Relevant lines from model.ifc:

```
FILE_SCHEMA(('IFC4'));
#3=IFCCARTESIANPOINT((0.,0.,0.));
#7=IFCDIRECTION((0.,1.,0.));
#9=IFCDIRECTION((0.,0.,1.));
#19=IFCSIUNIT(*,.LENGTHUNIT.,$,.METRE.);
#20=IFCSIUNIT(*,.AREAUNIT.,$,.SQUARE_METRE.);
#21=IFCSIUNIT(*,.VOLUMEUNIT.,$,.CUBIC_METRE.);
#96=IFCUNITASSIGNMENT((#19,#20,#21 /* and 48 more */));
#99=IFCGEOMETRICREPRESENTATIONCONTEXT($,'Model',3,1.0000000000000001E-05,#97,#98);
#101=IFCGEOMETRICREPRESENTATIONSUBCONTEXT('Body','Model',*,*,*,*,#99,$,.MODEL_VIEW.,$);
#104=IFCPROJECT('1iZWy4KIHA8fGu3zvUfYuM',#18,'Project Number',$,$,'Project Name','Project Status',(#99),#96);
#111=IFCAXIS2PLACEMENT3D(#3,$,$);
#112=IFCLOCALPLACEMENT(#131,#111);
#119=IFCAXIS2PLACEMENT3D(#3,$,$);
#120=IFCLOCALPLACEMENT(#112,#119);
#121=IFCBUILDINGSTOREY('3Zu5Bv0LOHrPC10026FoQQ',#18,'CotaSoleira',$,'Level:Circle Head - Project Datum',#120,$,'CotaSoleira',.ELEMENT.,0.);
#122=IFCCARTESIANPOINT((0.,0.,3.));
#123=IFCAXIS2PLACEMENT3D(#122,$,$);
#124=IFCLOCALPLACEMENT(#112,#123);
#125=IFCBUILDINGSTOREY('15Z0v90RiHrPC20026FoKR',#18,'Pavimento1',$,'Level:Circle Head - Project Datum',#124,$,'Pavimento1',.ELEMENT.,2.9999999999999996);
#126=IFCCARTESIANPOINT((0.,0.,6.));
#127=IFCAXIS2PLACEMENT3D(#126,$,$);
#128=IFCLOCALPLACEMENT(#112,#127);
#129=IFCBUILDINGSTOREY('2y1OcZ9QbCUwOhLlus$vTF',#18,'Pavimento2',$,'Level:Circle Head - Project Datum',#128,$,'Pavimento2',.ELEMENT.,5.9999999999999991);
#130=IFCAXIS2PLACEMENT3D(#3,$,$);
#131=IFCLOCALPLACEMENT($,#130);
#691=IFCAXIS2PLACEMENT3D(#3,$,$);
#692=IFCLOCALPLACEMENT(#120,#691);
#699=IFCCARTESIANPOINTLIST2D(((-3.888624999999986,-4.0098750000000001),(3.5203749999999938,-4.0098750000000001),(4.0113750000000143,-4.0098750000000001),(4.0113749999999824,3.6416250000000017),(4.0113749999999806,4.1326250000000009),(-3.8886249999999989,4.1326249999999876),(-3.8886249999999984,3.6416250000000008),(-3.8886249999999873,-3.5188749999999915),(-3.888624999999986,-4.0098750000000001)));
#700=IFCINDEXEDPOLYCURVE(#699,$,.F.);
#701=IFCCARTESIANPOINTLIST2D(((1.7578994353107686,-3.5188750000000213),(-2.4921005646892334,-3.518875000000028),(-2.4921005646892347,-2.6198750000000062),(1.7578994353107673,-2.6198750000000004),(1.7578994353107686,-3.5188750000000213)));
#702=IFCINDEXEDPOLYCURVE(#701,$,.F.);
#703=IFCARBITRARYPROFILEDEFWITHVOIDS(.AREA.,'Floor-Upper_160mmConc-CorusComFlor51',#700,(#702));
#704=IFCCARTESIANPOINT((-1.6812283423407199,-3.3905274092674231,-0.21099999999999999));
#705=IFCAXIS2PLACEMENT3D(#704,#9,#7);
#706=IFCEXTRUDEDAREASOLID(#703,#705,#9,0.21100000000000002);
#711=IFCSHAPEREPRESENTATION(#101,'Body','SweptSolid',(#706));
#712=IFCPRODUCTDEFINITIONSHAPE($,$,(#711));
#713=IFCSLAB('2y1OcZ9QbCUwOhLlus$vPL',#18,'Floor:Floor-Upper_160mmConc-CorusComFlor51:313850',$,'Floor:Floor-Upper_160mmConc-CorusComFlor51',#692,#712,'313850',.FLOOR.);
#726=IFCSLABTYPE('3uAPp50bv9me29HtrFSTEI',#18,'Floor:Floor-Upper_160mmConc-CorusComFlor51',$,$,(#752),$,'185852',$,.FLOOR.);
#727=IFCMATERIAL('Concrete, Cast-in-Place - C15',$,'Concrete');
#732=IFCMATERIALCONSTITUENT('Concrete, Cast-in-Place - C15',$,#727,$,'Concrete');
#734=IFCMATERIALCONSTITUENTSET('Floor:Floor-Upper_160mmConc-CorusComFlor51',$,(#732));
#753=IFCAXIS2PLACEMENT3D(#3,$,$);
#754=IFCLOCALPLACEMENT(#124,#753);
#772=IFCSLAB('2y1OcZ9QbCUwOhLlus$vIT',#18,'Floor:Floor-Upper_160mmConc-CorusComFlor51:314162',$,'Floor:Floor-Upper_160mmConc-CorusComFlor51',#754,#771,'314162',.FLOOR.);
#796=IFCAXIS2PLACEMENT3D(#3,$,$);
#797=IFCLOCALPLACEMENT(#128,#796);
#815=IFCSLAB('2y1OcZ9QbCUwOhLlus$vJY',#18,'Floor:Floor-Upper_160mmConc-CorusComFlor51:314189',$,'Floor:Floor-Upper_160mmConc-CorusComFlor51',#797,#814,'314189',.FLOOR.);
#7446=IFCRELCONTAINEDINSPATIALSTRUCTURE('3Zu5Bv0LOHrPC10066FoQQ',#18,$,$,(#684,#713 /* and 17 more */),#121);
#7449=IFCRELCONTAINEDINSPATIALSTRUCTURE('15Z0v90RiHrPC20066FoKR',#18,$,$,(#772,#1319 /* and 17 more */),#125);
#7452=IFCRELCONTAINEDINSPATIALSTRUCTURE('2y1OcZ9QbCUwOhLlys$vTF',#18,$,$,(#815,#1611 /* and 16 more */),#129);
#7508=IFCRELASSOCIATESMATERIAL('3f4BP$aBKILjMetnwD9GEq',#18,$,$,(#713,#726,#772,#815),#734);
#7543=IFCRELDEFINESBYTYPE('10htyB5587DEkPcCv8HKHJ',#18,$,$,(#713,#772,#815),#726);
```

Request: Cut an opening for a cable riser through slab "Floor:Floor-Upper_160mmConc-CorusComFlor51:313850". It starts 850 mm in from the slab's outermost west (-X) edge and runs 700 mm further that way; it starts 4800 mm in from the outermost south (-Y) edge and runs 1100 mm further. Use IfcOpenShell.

```python
import numpy as np
import ifcopenshell
import ifcopenshell.api.feature
import ifcopenshell.api.geometry
import ifcopenshell.api.root
import ifcopenshell.geom
import ifcopenshell.util.placement
import ifcopenshell.util.representation
import ifcopenshell.util.shape
import ifcopenshell.util.unit

model = ifcopenshell.open("model.ifc")
unit_scale = ifcopenshell.util.unit.calculate_unit_scale(model)
settings = ifcopenshell.geom.settings()


def volume(element):
    """Net volume in cubic metres, openings subtracted."""
    shape = ifcopenshell.geom.create_shape(settings, element)
    return ifcopenshell.util.shape.get_volume(shape.geometry)


slab = model.by_id(713)
before = volume(slab)

# Extent in the slab's own axes, in metres. The edges named are its -X and -Y sides.
slab_shape = ifcopenshell.geom.create_shape(settings, slab)
vertices = ifcopenshell.util.shape.get_vertices(slab_shape.geometry)
x_min, y_min, bottom = vertices.min(axis=0)
top = vertices[:, 2].max()

opening = ifcopenshell.api.root.create_entity(model, ifc_class="IfcOpeningElement", name="Cable riser opening", predefined_type="OPENING")
context = ifcopenshell.util.representation.get_context(model, "Model", "Body", "MODEL_VIEW")
width, depth = 0.7, 1.1
outline = [(0.0, 0.0), (width, 0.0), (width, depth), (0.0, depth), (0.0, 0.0)]
# Overshoot both faces by 50 mm so the cut is clean.
shape = ifcopenshell.api.geometry.add_slab_representation(
    model, context=context, depth=top - bottom + 0.1, polyline=outline
)
ifcopenshell.api.geometry.assign_representation(model, product=opening, representation=shape)

matrix = ifcopenshell.util.placement.get_local_placement(slab.ObjectPlacement)
matrix[:, 3] = matrix @ np.append(np.array([x_min + 0.85, y_min + 4.8, bottom - 0.05]) / unit_scale, 1.0)
ifcopenshell.api.geometry.edit_object_placement(model, product=opening, matrix=matrix, is_si=False)
ifcopenshell.api.feature.add_feature(model, feature=opening, element=slab)

after = volume(slab)

print(f"slab volume {before:.3f} -> {after:.3f} m3")

model.write("model-out.ifc")
```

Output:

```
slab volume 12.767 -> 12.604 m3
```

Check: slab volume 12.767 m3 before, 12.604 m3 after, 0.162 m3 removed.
